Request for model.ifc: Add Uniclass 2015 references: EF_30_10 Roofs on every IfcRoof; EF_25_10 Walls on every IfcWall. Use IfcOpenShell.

First a look at what the model holds.

```python
import ifcopenshell

model = ifcopenshell.open("model.ifc")
print(model.schema)
print("classifications:", [c.Name for c in model.by_type("IfcClassification")])
for ifc_class in ("IfcDoor", "IfcRoof", "IfcStair", "IfcWall", "IfcWindow"):
    print(ifc_class, len(model.by_type(ifc_class)))
```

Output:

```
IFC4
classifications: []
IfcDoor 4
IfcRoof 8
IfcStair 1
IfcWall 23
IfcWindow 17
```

```python
import ifcopenshell
import ifcopenshell.api.classification

model = ifcopenshell.open("model.ifc")

system = ifcopenshell.api.classification.add_classification(model, classification="Uniclass 2015")

codes = {
    "IfcRoof": ("EF_30_10", "Roofs"),
    "IfcWall": ("EF_25_10", "Walls"),
}
for ifc_class, (code, name) in codes.items():
    products = model.by_type(ifc_class)
    ifcopenshell.api.classification.add_reference(
        model, products=products, classification=system, identification=code, name=name
    )
    print(code, len(products))

model.write("model_edited.ifc")
```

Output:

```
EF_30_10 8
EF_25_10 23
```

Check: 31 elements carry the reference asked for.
